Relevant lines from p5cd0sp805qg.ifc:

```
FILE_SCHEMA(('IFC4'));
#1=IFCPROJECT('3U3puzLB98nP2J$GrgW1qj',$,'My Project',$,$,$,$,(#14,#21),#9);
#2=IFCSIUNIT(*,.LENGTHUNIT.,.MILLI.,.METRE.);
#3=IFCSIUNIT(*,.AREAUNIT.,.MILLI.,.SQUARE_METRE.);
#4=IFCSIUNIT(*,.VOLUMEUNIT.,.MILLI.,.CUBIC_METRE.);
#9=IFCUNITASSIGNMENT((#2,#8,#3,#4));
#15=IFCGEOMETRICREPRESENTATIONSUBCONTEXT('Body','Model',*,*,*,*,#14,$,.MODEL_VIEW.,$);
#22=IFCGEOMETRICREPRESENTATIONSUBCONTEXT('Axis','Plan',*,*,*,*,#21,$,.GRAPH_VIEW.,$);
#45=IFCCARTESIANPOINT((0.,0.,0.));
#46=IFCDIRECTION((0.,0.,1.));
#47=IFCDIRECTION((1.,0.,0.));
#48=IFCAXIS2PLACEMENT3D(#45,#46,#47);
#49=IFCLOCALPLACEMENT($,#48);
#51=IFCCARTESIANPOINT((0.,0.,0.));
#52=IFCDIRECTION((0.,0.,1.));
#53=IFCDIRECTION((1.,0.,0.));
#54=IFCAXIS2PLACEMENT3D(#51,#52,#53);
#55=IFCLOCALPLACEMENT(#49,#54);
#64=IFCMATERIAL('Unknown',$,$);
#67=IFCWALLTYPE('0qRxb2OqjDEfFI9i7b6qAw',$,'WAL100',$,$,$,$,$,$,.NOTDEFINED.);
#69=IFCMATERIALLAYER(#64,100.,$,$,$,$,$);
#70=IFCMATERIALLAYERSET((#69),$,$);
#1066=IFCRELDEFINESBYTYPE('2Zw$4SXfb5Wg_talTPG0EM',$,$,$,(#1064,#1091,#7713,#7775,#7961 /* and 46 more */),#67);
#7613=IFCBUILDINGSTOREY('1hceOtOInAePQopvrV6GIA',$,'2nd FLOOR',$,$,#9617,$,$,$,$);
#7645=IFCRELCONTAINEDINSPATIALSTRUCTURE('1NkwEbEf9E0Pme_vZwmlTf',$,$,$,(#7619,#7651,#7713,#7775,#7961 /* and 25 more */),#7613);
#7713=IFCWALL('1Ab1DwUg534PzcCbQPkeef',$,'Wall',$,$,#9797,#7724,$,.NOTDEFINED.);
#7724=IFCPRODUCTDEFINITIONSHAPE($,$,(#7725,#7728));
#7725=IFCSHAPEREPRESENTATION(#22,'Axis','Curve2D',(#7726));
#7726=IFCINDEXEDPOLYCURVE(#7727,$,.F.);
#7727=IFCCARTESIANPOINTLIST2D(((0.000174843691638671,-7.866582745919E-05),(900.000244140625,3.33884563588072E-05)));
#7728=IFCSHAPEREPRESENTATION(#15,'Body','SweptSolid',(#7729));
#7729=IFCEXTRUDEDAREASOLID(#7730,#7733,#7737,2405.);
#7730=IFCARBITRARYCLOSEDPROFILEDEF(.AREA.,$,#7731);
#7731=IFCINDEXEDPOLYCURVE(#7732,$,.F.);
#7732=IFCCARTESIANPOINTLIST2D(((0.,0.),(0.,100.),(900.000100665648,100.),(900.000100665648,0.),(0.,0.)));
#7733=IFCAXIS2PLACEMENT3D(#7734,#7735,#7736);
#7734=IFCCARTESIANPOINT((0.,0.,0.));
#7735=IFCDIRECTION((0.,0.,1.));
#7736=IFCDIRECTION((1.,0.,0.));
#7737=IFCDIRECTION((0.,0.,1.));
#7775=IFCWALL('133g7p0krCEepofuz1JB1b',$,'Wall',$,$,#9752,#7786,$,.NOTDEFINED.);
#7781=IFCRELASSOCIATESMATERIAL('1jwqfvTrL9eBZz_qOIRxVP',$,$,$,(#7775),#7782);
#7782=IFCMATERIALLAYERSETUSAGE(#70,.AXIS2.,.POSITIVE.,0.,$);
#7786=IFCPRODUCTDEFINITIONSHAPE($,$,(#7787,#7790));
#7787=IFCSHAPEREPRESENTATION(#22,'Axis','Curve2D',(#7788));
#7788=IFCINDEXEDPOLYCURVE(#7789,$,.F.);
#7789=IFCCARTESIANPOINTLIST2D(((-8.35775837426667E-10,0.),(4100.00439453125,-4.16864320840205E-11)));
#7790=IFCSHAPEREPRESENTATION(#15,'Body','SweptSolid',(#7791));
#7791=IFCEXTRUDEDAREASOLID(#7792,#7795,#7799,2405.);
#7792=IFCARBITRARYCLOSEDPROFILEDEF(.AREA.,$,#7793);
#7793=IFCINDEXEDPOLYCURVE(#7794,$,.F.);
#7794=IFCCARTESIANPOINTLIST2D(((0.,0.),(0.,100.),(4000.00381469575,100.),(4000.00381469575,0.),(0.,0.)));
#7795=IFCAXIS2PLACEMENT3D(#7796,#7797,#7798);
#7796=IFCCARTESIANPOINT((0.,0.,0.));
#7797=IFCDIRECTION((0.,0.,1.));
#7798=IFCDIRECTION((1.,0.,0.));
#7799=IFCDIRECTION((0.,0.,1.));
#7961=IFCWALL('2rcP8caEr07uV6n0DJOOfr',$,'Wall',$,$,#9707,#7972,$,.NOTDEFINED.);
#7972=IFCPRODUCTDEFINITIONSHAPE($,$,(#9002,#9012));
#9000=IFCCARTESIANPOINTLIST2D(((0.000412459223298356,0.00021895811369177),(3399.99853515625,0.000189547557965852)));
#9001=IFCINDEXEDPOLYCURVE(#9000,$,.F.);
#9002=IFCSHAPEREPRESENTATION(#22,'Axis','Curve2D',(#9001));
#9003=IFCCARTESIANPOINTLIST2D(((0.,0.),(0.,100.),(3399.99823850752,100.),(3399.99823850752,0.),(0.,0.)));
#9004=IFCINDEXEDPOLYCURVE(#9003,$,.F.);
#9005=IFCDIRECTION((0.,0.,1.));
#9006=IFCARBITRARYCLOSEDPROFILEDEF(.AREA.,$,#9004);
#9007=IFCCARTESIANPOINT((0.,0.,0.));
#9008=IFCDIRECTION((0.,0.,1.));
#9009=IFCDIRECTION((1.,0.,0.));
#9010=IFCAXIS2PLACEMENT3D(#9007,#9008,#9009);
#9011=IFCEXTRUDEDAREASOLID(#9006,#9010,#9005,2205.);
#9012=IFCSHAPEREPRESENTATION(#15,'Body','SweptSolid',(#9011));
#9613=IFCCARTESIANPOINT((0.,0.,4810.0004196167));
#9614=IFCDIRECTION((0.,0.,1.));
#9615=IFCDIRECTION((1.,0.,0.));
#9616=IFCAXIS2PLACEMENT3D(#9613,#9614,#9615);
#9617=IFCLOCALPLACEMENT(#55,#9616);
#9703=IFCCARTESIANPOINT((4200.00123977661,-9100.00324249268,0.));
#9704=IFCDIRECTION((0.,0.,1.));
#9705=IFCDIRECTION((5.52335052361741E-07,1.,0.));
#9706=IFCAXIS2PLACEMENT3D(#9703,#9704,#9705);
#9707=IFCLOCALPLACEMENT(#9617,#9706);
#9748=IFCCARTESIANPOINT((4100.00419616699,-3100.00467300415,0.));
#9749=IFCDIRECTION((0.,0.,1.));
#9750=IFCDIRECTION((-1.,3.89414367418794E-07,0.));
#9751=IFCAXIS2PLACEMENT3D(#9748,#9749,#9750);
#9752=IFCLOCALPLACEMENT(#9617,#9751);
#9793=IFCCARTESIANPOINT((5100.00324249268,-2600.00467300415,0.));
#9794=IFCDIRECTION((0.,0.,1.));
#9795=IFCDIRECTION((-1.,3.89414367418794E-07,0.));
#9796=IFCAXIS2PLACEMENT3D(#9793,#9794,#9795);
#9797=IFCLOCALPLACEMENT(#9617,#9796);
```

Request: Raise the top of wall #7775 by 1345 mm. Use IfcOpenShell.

```python
import ifcopenshell
import ifcopenshell.geom
import ifcopenshell.util.representation
import ifcopenshell.util.shape
import ifcopenshell.util.unit

model = ifcopenshell.open("p5cd0sp805qg.ifc")
unit_scale = ifcopenshell.util.unit.calculate_unit_scale(model)
settings = ifcopenshell.geom.settings()


def volume(element):
    """Net volume in cubic metres, openings subtracted."""
    shape = ifcopenshell.geom.create_shape(settings, element)
    return ifcopenshell.util.shape.get_volume(shape.geometry)


wall = model.by_guid("133g7p0krCEepofuz1JB1b")
before = volume(wall)

body = ifcopenshell.util.representation.get_representation(wall, "Model", "Body")
solid = body.Items[0]
old_height = solid.Depth
solid.Depth += 1.345 / unit_scale
after = volume(wall)

print(f"height {old_height:g} -> {solid.Depth:g}, volume {before:.3f} -> {after:.3f} m3")

model.write("p5cd0sp805qg_rev.ifc")
```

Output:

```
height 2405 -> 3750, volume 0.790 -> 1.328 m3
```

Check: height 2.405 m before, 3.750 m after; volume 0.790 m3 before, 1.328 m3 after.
